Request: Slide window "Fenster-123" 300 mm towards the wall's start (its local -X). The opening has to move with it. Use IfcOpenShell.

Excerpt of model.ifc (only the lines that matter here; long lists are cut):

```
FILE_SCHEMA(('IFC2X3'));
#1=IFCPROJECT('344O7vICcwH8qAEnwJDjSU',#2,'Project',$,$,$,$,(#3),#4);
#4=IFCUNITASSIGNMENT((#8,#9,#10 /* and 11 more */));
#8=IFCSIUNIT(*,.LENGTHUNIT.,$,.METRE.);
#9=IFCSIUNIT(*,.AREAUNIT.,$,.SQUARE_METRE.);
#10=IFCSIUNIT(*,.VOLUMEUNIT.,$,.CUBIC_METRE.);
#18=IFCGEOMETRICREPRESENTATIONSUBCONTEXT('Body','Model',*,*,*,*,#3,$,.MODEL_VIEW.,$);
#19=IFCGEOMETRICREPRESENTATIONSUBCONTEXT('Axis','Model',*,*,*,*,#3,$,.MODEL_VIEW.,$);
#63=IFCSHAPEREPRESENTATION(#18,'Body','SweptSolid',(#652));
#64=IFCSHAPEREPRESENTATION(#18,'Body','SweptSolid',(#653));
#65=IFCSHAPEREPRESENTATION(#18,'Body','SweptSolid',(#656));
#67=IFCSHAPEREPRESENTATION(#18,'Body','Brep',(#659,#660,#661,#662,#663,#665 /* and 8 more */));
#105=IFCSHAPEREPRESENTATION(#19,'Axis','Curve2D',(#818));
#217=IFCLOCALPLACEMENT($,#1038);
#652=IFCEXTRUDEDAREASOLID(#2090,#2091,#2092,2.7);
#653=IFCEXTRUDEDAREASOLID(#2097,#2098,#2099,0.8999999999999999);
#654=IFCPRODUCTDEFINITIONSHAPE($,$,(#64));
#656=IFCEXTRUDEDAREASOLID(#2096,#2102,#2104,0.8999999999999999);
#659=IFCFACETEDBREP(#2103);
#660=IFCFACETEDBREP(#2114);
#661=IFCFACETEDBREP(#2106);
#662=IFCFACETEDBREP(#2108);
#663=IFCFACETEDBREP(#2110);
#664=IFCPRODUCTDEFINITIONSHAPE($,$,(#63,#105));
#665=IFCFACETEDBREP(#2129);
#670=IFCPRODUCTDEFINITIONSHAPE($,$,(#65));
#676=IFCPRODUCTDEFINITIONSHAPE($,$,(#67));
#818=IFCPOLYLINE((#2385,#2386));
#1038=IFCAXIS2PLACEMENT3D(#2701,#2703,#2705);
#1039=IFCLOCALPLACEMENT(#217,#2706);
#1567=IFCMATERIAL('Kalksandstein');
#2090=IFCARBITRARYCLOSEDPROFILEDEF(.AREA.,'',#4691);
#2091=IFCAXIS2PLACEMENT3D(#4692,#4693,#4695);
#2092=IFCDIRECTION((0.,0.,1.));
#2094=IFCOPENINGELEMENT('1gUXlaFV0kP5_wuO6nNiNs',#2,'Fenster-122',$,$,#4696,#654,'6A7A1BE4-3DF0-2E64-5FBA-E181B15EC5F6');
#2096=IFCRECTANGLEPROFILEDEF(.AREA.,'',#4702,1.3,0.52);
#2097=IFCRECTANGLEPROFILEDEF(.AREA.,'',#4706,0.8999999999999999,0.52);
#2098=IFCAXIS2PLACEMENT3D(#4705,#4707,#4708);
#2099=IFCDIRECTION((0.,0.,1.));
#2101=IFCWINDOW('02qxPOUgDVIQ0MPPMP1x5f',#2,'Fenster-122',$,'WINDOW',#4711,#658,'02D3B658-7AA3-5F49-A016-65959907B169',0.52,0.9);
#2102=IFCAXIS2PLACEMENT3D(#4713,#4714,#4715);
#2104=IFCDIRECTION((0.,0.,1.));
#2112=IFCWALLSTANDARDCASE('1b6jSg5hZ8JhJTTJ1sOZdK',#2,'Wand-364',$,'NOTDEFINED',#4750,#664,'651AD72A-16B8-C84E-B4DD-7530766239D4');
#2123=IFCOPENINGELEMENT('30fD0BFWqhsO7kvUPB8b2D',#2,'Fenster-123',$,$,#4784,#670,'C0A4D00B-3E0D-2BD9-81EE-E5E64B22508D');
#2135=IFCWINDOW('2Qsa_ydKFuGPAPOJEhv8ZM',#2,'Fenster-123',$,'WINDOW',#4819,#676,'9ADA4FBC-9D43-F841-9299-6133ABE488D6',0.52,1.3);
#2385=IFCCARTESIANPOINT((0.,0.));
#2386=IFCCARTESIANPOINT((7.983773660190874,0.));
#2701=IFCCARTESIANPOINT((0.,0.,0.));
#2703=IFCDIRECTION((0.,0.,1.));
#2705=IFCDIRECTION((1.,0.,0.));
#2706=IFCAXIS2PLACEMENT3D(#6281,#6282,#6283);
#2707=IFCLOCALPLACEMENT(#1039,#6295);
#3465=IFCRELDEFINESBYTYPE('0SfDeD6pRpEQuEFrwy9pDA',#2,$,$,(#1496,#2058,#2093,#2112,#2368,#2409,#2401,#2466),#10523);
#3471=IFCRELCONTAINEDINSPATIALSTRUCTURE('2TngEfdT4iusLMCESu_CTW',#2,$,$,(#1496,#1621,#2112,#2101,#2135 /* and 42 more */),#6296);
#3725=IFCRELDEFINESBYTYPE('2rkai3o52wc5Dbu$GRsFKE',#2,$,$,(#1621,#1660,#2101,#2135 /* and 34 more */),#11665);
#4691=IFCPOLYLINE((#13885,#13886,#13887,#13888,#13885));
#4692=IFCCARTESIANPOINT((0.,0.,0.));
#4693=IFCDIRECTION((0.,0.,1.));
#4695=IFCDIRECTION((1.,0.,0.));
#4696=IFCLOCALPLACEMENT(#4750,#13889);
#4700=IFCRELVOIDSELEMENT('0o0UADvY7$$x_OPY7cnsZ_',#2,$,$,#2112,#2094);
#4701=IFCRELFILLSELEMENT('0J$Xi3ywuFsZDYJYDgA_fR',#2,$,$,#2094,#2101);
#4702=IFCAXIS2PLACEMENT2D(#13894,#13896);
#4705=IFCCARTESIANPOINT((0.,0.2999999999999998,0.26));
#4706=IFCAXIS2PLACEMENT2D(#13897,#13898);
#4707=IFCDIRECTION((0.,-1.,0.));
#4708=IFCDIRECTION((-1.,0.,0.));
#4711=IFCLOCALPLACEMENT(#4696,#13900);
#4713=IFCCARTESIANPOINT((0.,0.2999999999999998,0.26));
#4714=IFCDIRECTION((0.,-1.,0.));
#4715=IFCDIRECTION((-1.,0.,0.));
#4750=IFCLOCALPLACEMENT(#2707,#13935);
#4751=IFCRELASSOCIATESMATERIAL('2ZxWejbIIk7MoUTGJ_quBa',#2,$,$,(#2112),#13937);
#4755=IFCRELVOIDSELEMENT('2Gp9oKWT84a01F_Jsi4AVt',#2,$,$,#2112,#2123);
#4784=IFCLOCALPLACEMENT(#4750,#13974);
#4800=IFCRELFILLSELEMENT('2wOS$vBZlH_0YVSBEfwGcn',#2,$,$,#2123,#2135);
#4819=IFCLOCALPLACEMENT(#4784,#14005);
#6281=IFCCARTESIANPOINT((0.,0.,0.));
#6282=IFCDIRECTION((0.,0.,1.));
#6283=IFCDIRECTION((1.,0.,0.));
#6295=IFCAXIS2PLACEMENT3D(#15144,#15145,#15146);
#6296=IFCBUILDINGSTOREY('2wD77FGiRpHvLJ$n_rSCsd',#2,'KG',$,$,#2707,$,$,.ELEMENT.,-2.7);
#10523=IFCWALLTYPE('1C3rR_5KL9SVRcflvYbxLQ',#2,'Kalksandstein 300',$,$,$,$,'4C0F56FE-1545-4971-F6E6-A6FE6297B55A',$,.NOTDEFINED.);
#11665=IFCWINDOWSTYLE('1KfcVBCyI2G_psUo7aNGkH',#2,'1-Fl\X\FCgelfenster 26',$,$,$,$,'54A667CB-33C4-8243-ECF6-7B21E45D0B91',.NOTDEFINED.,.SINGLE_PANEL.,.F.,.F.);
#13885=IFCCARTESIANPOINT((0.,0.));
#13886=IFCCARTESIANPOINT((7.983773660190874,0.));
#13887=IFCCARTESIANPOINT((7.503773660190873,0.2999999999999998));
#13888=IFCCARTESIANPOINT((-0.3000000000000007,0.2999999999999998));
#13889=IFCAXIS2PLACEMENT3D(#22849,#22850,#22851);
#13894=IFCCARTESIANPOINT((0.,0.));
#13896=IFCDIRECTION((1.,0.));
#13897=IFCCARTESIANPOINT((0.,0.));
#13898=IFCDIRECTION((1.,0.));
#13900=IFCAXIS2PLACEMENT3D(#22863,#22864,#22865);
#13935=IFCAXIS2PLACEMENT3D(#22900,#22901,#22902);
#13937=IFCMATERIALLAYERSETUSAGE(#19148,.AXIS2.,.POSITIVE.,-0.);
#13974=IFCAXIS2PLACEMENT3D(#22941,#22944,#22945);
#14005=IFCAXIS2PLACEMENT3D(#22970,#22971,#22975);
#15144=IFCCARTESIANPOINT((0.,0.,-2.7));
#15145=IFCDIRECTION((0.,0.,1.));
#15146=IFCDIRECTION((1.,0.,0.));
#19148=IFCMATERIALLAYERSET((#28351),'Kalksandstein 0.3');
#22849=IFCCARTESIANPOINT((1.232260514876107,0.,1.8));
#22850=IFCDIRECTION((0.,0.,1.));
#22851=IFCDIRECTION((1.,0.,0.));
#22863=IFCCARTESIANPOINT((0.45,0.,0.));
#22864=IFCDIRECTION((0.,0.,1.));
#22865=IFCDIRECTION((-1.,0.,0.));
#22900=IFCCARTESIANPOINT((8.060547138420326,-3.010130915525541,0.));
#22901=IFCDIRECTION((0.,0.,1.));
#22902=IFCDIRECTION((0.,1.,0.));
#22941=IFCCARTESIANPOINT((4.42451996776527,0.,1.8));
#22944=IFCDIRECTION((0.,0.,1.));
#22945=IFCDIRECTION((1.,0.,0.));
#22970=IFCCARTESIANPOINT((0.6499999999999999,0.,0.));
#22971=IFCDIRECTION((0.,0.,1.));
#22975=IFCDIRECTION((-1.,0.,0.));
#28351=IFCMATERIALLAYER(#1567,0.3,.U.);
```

```python
import ifcopenshell
import ifcopenshell.api.geometry
import ifcopenshell.util.placement
import ifcopenshell.util.unit

model = ifcopenshell.open("model.ifc")
unit_scale = ifcopenshell.util.unit.calculate_unit_scale(model)

window = model.by_guid("2Qsa_ydKFuGPAPOJEhv8ZM")
opening = window.FillsVoids[0].RelatingOpeningElement
wall = opening.VoidsElements[0].RelatingBuildingElement

wall_matrix = ifcopenshell.util.placement.get_local_placement(wall.ObjectPlacement)
shift = wall_matrix[:3, 0] * -0.3 / unit_scale
before = ifcopenshell.util.placement.get_local_placement(window.ObjectPlacement)[:3, 3].copy()

# The window is placed relative to its opening, so it follows when the opening moves.
matrix = ifcopenshell.util.placement.get_local_placement(opening.ObjectPlacement)
matrix[:3, 3] += shift
ifcopenshell.api.geometry.edit_object_placement(
    model, product=opening, matrix=matrix, is_si=False, should_transform_children=True
)

after = ifcopenshell.util.placement.get_local_placement(window.ObjectPlacement)[:3, 3]
print("window moved by", (after - before).round(3) + 0.0)

model.write("model_edited.ifc")
```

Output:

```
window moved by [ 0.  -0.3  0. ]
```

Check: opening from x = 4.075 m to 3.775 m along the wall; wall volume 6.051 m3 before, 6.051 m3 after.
